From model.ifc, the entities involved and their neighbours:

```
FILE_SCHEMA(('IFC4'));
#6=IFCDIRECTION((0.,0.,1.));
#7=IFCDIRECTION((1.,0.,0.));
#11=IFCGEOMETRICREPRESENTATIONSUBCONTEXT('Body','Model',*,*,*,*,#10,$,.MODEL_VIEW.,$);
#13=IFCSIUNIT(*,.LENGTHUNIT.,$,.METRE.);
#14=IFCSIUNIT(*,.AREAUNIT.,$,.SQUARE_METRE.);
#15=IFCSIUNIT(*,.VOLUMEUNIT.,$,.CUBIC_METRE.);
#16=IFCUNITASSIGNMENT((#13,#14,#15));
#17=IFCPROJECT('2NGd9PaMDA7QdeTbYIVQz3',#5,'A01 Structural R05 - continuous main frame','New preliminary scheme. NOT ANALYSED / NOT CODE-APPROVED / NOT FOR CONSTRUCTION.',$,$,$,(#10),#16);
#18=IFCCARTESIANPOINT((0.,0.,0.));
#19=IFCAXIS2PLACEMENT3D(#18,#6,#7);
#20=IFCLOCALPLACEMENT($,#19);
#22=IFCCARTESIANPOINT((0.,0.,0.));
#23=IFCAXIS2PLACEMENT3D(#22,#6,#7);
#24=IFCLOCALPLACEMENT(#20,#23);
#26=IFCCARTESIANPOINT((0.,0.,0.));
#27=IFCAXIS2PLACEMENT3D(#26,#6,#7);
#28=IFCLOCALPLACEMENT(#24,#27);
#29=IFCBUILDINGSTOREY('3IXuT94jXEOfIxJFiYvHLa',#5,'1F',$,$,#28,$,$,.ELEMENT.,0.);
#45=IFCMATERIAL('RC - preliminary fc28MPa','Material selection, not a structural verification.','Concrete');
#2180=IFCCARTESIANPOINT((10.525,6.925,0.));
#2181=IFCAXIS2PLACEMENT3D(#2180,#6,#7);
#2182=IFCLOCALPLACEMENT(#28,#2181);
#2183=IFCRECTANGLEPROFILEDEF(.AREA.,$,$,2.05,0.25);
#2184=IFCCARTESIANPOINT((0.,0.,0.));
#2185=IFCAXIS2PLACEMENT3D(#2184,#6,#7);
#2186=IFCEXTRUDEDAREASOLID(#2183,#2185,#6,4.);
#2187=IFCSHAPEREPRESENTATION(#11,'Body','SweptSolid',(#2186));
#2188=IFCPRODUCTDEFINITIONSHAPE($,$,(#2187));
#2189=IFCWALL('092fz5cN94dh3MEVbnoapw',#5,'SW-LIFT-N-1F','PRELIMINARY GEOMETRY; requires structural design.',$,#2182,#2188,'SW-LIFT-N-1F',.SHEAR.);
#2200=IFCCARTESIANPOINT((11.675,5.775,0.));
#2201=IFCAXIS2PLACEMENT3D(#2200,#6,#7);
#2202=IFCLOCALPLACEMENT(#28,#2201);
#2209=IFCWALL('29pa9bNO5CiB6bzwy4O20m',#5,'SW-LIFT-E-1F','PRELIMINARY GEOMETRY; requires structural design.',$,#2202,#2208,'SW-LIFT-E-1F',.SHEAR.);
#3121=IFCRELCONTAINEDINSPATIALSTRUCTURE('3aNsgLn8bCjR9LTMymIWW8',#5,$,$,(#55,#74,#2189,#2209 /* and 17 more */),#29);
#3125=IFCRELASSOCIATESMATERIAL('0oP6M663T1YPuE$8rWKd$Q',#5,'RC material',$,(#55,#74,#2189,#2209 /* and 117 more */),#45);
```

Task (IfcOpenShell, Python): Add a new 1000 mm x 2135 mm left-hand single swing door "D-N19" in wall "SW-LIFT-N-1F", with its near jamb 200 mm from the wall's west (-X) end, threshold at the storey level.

```python
import numpy as np
import ifcopenshell
import ifcopenshell.api.feature
import ifcopenshell.api.geometry
import ifcopenshell.api.root
import ifcopenshell.api.spatial
import ifcopenshell.geom
import ifcopenshell.util.element
import ifcopenshell.util.placement
import ifcopenshell.util.representation
import ifcopenshell.util.shape
import ifcopenshell.util.unit

model = ifcopenshell.open("model.ifc")
unit_scale = ifcopenshell.util.unit.calculate_unit_scale(model)
settings = ifcopenshell.geom.settings()


def volume(element):
    """Net volume in cubic metres, openings subtracted."""
    shape = ifcopenshell.geom.create_shape(settings, element)
    return ifcopenshell.util.shape.get_volume(shape.geometry)


wall = model.by_guid("092fz5cN94dh3MEVbnoapw")
storey = ifcopenshell.util.element.get_container(wall, ifc_class="IfcBuildingStorey")
context = ifcopenshell.util.representation.get_context(model, "Model", "Body", "MODEL_VIEW")
before = volume(wall)

width, height, from_end, sill = 1, 2.135, 0.2, 0.0  # metres

# The wall runs along its own X axis, and the end named is its -X end.
wall_shape = ifcopenshell.geom.create_shape(settings, wall)
x, y, z = ifcopenshell.util.shape.get_vertices(wall_shape.geometry).T
start = x.min() + from_end
face, thickness = float(y.min()), float(y.max() - y.min())
wall_matrix = ifcopenshell.util.placement.get_local_placement(wall.ObjectPlacement)
level = ifcopenshell.util.placement.get_local_placement(storey.ObjectPlacement)[2, 3]


def in_wall(x, y):
    """Placement at x, y metres in the wall's axes, at sill height."""
    matrix = wall_matrix.copy()
    matrix[:, 3] = wall_matrix @ np.array([x / unit_scale, y / unit_scale, 0.0, 1.0])
    matrix[2, 3] = level + sill / unit_scale
    return matrix


# Opening: a box that overshoots both wall faces by 50 mm.
opening = ifcopenshell.api.root.create_entity(model, ifc_class="IfcOpeningElement", predefined_type="OPENING")
box = ifcopenshell.api.geometry.add_wall_representation(
    model, context=context, length=width, height=height, thickness=thickness + 0.1
)
ifcopenshell.api.geometry.assign_representation(model, product=opening, representation=box)
ifcopenshell.api.geometry.edit_object_placement(model, product=opening, matrix=in_wall(start, face - 0.05), is_si=False)
ifcopenshell.api.feature.add_feature(model, feature=opening, element=wall)

door = ifcopenshell.api.root.create_entity(model, ifc_class="IfcDoor", name="D-N19", predefined_type="DOOR")
door.OverallWidth, door.OverallHeight = width / unit_scale, height / unit_scale
door.OperationType = "SINGLE_SWING_LEFT"
body = ifcopenshell.api.geometry.add_door_representation(
    model,
    context=context,
    overall_width=door.OverallWidth,
    overall_height=door.OverallHeight,
    operation_type="SINGLE_SWING_LEFT",
    lining_properties={"LiningDepth": thickness / unit_scale, "ThresholdDepth": thickness / unit_scale},
)
ifcopenshell.api.geometry.assign_representation(model, product=door, representation=body)
ifcopenshell.api.spatial.assign_container(model, products=[door], relating_structure=storey)
ifcopenshell.api.feature.add_filling(model, opening=opening, element=door)

# The lining spans the wall, so the door starts at the wall face.
ifcopenshell.api.geometry.edit_object_placement(model, product=door, matrix=in_wall(start, face), is_si=False)

after = volume(wall)

print(f"wall volume {before:.3f} -> {after:.3f} m3")

model.write("model_v2.ifc")
```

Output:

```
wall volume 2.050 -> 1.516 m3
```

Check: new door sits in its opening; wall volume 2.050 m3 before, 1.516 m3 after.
